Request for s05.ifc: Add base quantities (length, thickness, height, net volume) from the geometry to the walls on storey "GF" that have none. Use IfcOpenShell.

First a look at what the model holds.

```python
import ifcopenshell
import ifcopenshell.util.element
import ifcopenshell.util.unit

model = ifcopenshell.open("s05.ifc")
print(model.schema)
for unit_type in ("LENGTHUNIT", "AREAUNIT", "VOLUMEUNIT"):
    print(unit_type, ifcopenshell.util.unit.calculate_unit_scale(model, unit_type))
storey = next(s for s in model.by_type("IfcBuildingStorey") if s.Name == "GF")
walls = [e for e in ifcopenshell.util.element.get_decomposition(storey) if e.is_a("IfcWall")]
for e in sorted(walls, key=lambda e: e.id()):
    print(e.id(), e.is_a(), e.Name, list(ifcopenshell.util.element.get_psets(e, qtos_only=True)), sep=" | ")
```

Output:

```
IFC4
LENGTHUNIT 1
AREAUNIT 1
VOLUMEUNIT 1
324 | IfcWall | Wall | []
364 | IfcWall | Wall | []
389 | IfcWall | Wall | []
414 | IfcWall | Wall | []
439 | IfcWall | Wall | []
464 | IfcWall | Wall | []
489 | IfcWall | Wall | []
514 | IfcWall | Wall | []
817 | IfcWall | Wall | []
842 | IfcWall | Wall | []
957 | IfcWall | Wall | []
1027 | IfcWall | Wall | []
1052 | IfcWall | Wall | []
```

```python
import ifcopenshell
import ifcopenshell.api.pset
import ifcopenshell.geom
import ifcopenshell.util.element
import ifcopenshell.util.shape
import ifcopenshell.util.unit

model = ifcopenshell.open("s05.ifc")
unit_scale = ifcopenshell.util.unit.calculate_unit_scale(model)
volume_scale = ifcopenshell.util.unit.calculate_unit_scale(model, "VOLUMEUNIT")
settings = ifcopenshell.geom.settings()

storey = next(s for s in model.by_type("IfcBuildingStorey") if s.Name == "GF")
walls = [e for e in ifcopenshell.util.element.get_decomposition(storey) if e.is_a("IfcWall")]

for e in sorted(walls, key=lambda e: e.id()):
    if ifcopenshell.util.element.get_psets(e, qtos_only=True, should_inherit=False):
        continue
    # Geometry comes back in metres, in the element's own axes.
    shape = ifcopenshell.geom.create_shape(settings, e)
    values = {
        "Length": ifcopenshell.util.shape.get_x(shape.geometry) / unit_scale,
        "Width": ifcopenshell.util.shape.get_y(shape.geometry) / unit_scale,
        "Height": ifcopenshell.util.shape.get_z(shape.geometry) / unit_scale,
        "NetVolume": ifcopenshell.util.shape.get_volume(shape.geometry) / volume_scale,
    }
    qto = ifcopenshell.api.pset.add_qto(model, product=e, name="Qto_WallBaseQuantities")
    ifcopenshell.api.pset.edit_qto(model, qto=qto, properties=values)
    print(e.id(), {k: round(v, 3) for k, v in values.items()})

model.write("s05-out.ifc")
```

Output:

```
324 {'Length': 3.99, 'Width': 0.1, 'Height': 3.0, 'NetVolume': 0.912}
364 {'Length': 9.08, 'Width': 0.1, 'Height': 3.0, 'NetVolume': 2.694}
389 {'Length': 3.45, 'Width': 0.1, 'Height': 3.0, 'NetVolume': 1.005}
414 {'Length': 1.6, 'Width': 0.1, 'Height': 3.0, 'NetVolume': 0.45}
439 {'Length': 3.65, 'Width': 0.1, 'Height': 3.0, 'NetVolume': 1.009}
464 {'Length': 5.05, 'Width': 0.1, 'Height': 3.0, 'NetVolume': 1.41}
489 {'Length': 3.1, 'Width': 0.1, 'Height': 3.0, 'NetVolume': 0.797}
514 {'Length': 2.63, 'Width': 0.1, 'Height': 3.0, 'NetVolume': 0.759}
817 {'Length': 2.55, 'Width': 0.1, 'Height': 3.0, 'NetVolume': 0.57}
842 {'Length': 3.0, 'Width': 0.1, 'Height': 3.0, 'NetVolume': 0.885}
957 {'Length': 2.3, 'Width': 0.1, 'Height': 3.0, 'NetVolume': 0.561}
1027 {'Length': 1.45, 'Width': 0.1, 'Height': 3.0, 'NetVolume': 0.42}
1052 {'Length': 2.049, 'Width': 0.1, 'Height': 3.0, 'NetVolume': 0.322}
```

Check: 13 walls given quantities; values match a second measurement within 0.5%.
